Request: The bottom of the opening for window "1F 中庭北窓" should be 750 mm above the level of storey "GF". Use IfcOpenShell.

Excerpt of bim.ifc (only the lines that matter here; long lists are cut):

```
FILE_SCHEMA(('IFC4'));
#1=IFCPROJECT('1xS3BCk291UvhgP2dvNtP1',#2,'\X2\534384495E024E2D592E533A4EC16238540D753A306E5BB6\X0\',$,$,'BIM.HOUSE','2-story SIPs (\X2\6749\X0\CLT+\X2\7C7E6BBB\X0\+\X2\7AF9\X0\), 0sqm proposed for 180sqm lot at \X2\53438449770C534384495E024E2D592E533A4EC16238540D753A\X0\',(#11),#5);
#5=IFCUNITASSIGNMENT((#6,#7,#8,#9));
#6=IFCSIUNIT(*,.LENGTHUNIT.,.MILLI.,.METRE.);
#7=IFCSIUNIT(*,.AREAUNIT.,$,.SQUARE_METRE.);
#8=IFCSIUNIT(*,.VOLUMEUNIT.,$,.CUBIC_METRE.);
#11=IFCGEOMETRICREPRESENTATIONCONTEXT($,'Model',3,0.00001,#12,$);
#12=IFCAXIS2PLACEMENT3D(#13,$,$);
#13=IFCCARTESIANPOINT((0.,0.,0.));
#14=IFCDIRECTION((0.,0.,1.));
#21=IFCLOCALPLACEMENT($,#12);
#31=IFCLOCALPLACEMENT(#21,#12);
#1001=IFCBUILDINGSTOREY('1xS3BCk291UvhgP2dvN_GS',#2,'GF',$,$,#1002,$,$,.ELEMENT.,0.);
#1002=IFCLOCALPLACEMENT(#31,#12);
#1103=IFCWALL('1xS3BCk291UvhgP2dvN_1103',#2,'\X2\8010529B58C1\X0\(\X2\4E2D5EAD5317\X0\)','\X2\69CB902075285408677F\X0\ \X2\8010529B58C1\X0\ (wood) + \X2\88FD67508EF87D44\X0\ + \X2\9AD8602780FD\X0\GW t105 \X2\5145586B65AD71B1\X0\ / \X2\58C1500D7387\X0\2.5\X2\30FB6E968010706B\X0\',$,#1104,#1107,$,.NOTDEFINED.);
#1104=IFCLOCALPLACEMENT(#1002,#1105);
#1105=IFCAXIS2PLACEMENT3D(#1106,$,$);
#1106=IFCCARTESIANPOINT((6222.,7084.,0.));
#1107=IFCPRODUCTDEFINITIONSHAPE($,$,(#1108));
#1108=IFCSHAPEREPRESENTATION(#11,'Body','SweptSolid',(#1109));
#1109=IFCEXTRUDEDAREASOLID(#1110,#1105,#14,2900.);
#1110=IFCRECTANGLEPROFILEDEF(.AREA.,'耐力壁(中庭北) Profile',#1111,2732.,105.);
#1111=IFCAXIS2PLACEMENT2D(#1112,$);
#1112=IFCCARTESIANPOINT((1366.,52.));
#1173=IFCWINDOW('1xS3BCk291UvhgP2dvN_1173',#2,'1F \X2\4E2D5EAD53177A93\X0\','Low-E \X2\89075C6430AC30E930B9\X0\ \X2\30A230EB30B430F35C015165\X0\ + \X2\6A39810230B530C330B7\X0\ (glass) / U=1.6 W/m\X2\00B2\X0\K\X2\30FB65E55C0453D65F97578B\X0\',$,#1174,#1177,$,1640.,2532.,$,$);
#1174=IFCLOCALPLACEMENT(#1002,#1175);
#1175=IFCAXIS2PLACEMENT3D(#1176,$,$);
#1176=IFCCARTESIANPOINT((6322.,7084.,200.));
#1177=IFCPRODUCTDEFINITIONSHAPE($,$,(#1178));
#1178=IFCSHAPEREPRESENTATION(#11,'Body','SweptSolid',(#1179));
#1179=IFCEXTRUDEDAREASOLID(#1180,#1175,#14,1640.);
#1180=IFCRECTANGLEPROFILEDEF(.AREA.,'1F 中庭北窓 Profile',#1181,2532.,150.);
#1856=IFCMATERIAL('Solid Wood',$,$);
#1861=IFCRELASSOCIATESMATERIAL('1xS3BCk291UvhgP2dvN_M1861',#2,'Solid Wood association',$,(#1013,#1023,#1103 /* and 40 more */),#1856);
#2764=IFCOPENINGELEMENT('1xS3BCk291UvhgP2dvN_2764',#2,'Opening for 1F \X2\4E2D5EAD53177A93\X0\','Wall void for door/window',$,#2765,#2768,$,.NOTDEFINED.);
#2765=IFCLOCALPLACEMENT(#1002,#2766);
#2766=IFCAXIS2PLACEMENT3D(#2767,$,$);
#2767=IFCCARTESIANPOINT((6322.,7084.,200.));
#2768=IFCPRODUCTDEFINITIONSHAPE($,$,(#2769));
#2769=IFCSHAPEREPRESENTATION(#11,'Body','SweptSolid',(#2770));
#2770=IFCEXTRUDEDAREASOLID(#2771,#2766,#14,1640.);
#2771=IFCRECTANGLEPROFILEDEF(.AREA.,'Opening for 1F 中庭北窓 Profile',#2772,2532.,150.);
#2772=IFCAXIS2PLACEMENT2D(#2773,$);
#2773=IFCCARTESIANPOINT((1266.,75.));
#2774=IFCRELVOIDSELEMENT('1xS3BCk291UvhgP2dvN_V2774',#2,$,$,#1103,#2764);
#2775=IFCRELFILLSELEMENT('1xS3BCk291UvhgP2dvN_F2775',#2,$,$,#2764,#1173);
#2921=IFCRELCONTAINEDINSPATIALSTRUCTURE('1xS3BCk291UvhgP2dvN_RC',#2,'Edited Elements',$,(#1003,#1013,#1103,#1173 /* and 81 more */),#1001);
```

```python
import numpy as np
import ifcopenshell
import ifcopenshell.api.geometry
import ifcopenshell.geom
import ifcopenshell.util.element
import ifcopenshell.util.placement
import ifcopenshell.util.shape
import ifcopenshell.util.unit

model = ifcopenshell.open("bim.ifc")
unit_scale = ifcopenshell.util.unit.calculate_unit_scale(model)

window = model.by_guid("1xS3BCk291UvhgP2dvN_1173")
opening = window.FillsVoids[0].RelatingOpeningElement
storey = ifcopenshell.util.element.get_container(window, ifc_class="IfcBuildingStorey")
level = ifcopenshell.util.placement.get_local_placement(storey.ObjectPlacement)[2, 3]

# The opening's origin need not be at the sill, so measure its lowest point.
shape = ifcopenshell.geom.create_shape(ifcopenshell.geom.settings(), opening)
bottom = ifcopenshell.util.shape.get_shape_bottom_elevation(shape, shape.geometry) / unit_scale
dz = level + 0.75 / unit_scale - bottom

shift = np.array([0.0, 0.0, dz])
# The window is not placed relative to its opening, so move both.
for product in (opening, window):
    matrix = ifcopenshell.util.placement.get_local_placement(product.ObjectPlacement)
    matrix[:3, 3] += shift
    ifcopenshell.api.geometry.edit_object_placement(model, product=product, matrix=matrix, is_si=False)

print(f"moved by {dz * unit_scale:+.3f} m")

model.write("bim_rev.ifc")
```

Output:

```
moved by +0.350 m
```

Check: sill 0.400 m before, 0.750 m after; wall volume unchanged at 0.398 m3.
